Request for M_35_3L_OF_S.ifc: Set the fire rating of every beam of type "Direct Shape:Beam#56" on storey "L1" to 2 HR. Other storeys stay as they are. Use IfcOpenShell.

First a look at what the model holds.

```python
import ifcopenshell
import ifcopenshell.util.element

model = ifcopenshell.open("M_35_3L_OF_S.ifc")
print(model.schema)
storey = next(s for s in model.by_type("IfcBuildingStorey") if s.Name == "L1")
beams = [e for e in ifcopenshell.util.element.get_decomposition(storey) if e.is_a("IfcBeam")]
seen = {}
for e in beams:
    element_type = ifcopenshell.util.element.get_type(e)
    key = (element_type.Name if element_type != e and element_type else None, ifcopenshell.util.element.get_pset(e, "Pset_BeamCommon", "FireRating"))
    seen[key] = seen.get(key, 0) + 1
for (name, value), count in sorted(seen.items(), key=str):
    print(count, "x", name, "|", value)
```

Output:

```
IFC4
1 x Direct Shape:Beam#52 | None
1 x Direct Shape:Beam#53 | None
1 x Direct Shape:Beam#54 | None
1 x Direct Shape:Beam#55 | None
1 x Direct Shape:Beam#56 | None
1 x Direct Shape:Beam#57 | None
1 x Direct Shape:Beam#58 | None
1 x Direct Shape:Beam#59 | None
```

```python
import ifcopenshell
import ifcopenshell.api.pset
import ifcopenshell.util.element

model = ifcopenshell.open("M_35_3L_OF_S.ifc")

storey = next(s for s in model.by_type("IfcBuildingStorey") if s.Name == "L1")
beams = [e for e in ifcopenshell.util.element.get_decomposition(storey) if e.is_a("IfcBeam")]

count = 0
for e in beams:
    element_type = ifcopenshell.util.element.get_type(e)
    if element_type in (None, e) or element_type.Name != "Direct Shape:Beam#56":
        continue
    # add_pset returns the element's existing set when there is one.
    pset = ifcopenshell.api.pset.add_pset(model, product=e, name="Pset_BeamCommon")
    ifcopenshell.api.pset.edit_pset(model, pset=pset, properties={"FireRating": "2 HR"})
    count += 1

print(count, "beams updated")

model.write("M_35_3L_OF_S_rev.ifc")
```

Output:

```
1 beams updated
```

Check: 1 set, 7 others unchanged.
